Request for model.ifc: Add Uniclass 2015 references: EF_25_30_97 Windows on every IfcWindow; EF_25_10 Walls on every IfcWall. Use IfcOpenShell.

First a look at what the model holds.

```python
import ifcopenshell

model = ifcopenshell.open("model.ifc")
print(model.schema)
print("classifications:", [c.Name for c in model.by_type("IfcClassification")])
for ifc_class in ("IfcDoor", "IfcRoof", "IfcStair", "IfcWall", "IfcWindow"):
    print(ifc_class, len(model.by_type(ifc_class)))
```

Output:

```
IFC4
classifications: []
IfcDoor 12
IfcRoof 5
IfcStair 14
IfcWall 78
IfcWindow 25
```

```python
import ifcopenshell
import ifcopenshell.api.classification

model = ifcopenshell.open("model.ifc")

system = ifcopenshell.api.classification.add_classification(model, classification="Uniclass 2015")

codes = {
    "IfcWindow": ("EF_25_30_97", "Windows"),
    "IfcWall": ("EF_25_10", "Walls"),
}
for ifc_class, (code, name) in codes.items():
    products = model.by_type(ifc_class)
    ifcopenshell.api.classification.add_reference(
        model, products=products, classification=system, identification=code, name=name
    )
    print(code, len(products))

model.write("model-out.ifc")
```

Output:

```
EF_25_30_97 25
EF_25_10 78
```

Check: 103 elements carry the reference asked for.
